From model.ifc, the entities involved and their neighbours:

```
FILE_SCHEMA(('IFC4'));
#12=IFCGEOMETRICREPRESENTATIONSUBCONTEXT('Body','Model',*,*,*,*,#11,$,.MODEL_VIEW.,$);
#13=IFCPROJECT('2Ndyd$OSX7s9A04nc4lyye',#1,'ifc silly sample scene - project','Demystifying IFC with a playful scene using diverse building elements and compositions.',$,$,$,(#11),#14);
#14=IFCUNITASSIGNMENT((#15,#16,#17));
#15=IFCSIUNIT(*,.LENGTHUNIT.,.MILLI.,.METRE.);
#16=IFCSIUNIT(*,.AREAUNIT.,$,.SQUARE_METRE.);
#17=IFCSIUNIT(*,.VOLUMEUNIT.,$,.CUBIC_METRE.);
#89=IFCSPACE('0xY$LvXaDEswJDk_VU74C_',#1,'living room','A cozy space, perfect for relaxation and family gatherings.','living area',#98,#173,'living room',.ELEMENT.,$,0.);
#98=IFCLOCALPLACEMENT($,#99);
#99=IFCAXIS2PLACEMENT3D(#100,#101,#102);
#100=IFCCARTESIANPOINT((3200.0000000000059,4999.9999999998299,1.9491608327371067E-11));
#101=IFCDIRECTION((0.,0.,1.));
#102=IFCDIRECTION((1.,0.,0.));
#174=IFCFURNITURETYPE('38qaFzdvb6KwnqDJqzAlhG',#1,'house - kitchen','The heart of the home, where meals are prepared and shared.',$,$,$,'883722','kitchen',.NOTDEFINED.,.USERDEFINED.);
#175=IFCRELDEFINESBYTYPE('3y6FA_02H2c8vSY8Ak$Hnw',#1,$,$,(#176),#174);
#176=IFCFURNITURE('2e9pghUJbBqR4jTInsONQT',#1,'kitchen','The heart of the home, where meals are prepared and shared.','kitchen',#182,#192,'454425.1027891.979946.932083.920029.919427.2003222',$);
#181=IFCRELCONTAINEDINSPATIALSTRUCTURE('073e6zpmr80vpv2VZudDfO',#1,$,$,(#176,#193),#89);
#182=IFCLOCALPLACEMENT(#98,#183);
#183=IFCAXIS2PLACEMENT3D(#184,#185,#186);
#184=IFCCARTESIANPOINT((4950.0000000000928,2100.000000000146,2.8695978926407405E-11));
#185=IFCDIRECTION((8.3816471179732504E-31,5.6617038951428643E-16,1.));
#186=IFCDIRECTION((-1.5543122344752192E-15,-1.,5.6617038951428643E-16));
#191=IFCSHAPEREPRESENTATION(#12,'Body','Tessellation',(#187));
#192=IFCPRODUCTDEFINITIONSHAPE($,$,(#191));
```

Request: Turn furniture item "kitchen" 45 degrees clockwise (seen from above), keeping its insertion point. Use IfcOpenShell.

```python
import ifcopenshell
import ifcopenshell.api.geometry
import ifcopenshell.util.placement

model = ifcopenshell.open("model.ifc")

item = model.by_guid("2e9pghUJbBqR4jTInsONQT")
matrix = ifcopenshell.util.placement.get_local_placement(item.ObjectPlacement)
matrix = matrix @ ifcopenshell.util.placement.rotation(-45, "Z")
ifcopenshell.api.geometry.edit_object_placement(model, product=item, matrix=matrix, is_si=False)

print(ifcopenshell.util.placement.get_local_placement(item.ObjectPlacement).round(3) + 0.0)

model.write("model-out.ifc")
```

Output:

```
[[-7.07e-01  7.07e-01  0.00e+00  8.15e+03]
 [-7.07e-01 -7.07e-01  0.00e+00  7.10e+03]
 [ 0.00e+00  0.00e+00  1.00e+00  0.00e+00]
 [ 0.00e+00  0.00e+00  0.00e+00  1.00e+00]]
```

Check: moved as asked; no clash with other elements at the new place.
